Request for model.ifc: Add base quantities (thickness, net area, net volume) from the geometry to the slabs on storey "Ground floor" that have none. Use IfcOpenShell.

First a look at what the model holds.

```python
import ifcopenshell
import ifcopenshell.util.element
import ifcopenshell.util.unit

model = ifcopenshell.open("model.ifc")
print(model.schema)
for unit_type in ("LENGTHUNIT", "AREAUNIT", "VOLUMEUNIT"):
    print(unit_type, ifcopenshell.util.unit.calculate_unit_scale(model, unit_type))
storey = next(s for s in model.by_type("IfcBuildingStorey") if s.Name == "Ground floor")
slabs = [e for e in ifcopenshell.util.element.get_decomposition(storey) if e.is_a("IfcSlab")]
for e in sorted(slabs, key=lambda e: e.id()):
    print(e.id(), e.is_a(), e.Name, list(ifcopenshell.util.element.get_psets(e, qtos_only=True)), sep=" | ")
```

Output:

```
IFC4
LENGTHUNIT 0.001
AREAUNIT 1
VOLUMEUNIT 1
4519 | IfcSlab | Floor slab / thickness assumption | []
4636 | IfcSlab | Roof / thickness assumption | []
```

```python
import ifcopenshell
import ifcopenshell.api.pset
import ifcopenshell.geom
import ifcopenshell.util.element
import ifcopenshell.util.shape
import ifcopenshell.util.unit

model = ifcopenshell.open("model.ifc")
unit_scale = ifcopenshell.util.unit.calculate_unit_scale(model)
area_scale = ifcopenshell.util.unit.calculate_unit_scale(model, "AREAUNIT")
volume_scale = ifcopenshell.util.unit.calculate_unit_scale(model, "VOLUMEUNIT")
settings = ifcopenshell.geom.settings()

storey = next(s for s in model.by_type("IfcBuildingStorey") if s.Name == "Ground floor")
slabs = [e for e in ifcopenshell.util.element.get_decomposition(storey) if e.is_a("IfcSlab")]

for e in sorted(slabs, key=lambda e: e.id()):
    if ifcopenshell.util.element.get_psets(e, qtos_only=True, should_inherit=False):
        continue
    # Geometry comes back in metres, in the element's own axes.
    shape = ifcopenshell.geom.create_shape(settings, e)
    values = {
        "Width": ifcopenshell.util.shape.get_z(shape.geometry) / unit_scale,
        "NetArea": ifcopenshell.util.shape.get_footprint_area(shape.geometry) / area_scale,
        "NetVolume": ifcopenshell.util.shape.get_volume(shape.geometry) / volume_scale,
    }
    qto = ifcopenshell.api.pset.add_qto(model, product=e, name="Qto_SlabBaseQuantities")
    ifcopenshell.api.pset.edit_qto(model, qto=qto, properties=values)
    print(e.id(), {k: round(v, 3) for k, v in values.items()})

model.write("model_rev.ifc")
```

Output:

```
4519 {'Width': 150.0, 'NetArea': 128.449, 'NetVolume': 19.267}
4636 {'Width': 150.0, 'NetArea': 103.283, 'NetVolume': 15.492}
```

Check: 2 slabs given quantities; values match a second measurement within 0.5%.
